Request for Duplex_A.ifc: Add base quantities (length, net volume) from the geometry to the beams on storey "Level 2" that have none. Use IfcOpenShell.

First a look at what the model holds.

```python
import ifcopenshell
import ifcopenshell.util.element
import ifcopenshell.util.unit

model = ifcopenshell.open("Duplex_A.ifc")
print(model.schema)
for unit_type in ("LENGTHUNIT", "AREAUNIT", "VOLUMEUNIT"):
    print(unit_type, ifcopenshell.util.unit.calculate_unit_scale(model, unit_type))
storey = next(s for s in model.by_type("IfcBuildingStorey") if s.Name == "Level 2")
beams = [e for e in ifcopenshell.util.element.get_decomposition(storey) if e.is_a("IfcBeam")]
for e in sorted(beams, key=lambda e: e.id()):
    print(e.id(), e.is_a(), e.Name, list(ifcopenshell.util.element.get_psets(e, qtos_only=True)), sep=" | ")
```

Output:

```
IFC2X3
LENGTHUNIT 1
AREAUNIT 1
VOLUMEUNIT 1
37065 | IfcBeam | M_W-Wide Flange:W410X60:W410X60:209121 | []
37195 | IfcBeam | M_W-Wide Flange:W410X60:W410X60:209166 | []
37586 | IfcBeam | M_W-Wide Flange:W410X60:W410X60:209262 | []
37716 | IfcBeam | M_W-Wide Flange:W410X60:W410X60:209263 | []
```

```python
import ifcopenshell
import ifcopenshell.api.pset
import ifcopenshell.geom
import ifcopenshell.util.element
import ifcopenshell.util.shape
import ifcopenshell.util.unit

model = ifcopenshell.open("Duplex_A.ifc")
unit_scale = ifcopenshell.util.unit.calculate_unit_scale(model)
volume_scale = ifcopenshell.util.unit.calculate_unit_scale(model, "VOLUMEUNIT")
settings = ifcopenshell.geom.settings()

storey = next(s for s in model.by_type("IfcBuildingStorey") if s.Name == "Level 2")
beams = [e for e in ifcopenshell.util.element.get_decomposition(storey) if e.is_a("IfcBeam")]

for e in sorted(beams, key=lambda e: e.id()):
    if ifcopenshell.util.element.get_psets(e, qtos_only=True, should_inherit=False):
        continue
    # Geometry comes back in metres, in the element's own axes.
    shape = ifcopenshell.geom.create_shape(settings, e)
    values = {
        "Length": ifcopenshell.util.shape.get_max_xyz(shape.geometry) / unit_scale,
        "NetVolume": ifcopenshell.util.shape.get_volume(shape.geometry) / volume_scale,
    }
    qto = ifcopenshell.api.pset.add_qto(model, product=e, name="BaseQuantities")
    ifcopenshell.api.pset.edit_qto(model, qto=qto, properties=values)
    print(e.id(), {k: round(v, 3) for k, v in values.items()})

model.write("Duplex_A_v2.ifc")
```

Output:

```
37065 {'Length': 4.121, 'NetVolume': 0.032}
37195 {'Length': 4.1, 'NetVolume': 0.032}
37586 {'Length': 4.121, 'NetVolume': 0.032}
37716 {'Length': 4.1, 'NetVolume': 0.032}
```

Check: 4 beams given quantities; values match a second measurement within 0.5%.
